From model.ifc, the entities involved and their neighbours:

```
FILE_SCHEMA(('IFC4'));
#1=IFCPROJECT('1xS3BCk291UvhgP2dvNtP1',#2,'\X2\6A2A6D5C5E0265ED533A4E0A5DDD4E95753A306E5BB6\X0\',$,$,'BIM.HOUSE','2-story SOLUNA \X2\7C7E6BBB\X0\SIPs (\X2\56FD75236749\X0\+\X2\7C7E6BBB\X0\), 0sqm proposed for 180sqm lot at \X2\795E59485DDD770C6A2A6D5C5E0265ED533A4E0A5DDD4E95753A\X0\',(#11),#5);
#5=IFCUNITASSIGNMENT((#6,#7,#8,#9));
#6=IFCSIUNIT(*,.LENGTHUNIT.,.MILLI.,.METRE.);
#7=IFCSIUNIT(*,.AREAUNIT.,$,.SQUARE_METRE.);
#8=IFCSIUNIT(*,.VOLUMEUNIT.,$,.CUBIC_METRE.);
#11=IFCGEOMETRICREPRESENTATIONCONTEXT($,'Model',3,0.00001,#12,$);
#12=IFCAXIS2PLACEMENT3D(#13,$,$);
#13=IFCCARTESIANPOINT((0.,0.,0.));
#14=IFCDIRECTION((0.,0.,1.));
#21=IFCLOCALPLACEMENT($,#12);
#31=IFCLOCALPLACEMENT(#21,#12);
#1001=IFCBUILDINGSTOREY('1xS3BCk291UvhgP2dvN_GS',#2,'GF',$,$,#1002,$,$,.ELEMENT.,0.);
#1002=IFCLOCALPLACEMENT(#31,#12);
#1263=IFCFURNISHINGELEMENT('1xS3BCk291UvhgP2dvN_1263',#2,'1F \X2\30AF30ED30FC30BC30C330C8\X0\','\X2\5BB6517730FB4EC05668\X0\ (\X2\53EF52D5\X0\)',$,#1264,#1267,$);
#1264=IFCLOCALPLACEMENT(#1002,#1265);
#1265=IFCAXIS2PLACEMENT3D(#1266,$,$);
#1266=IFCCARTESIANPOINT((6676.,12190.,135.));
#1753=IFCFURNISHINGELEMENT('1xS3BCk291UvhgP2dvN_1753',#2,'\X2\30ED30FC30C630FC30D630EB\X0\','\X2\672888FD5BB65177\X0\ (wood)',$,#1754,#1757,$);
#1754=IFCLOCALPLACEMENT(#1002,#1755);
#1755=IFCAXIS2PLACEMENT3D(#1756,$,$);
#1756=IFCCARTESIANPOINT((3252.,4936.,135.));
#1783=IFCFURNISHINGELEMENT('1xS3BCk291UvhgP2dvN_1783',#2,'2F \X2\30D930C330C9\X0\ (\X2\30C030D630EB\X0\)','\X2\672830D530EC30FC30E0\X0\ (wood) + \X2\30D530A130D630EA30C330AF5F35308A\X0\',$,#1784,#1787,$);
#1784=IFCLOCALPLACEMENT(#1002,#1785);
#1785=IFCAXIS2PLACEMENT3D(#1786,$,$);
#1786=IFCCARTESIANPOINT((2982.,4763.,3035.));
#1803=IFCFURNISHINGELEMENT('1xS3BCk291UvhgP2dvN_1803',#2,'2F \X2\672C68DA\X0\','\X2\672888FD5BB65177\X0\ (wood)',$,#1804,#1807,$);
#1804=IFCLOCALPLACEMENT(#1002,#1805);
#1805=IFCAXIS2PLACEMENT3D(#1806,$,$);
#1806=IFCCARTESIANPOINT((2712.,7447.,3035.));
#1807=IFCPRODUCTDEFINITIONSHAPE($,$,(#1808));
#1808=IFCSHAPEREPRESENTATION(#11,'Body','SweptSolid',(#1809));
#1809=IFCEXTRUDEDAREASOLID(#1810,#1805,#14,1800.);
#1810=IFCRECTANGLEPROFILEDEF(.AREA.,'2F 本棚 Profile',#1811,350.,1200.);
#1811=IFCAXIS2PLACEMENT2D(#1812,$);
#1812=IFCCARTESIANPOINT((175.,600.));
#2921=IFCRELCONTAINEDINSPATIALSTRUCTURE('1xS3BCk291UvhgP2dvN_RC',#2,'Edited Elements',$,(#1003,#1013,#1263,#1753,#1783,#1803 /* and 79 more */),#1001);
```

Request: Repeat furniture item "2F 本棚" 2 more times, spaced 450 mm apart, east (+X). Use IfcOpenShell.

```python
import numpy as np
import ifcopenshell
import ifcopenshell.api.geometry
import ifcopenshell.api.root
import ifcopenshell.util.element
import ifcopenshell.util.placement
import ifcopenshell.util.unit

model = ifcopenshell.open("model.ifc")
unit_scale = ifcopenshell.util.unit.calculate_unit_scale(model)


def reuse_history(source, copy):
    """copy_class also copies each property set's owner history, people and application; keep the originals."""
    for rel in copy.IsDefinedBy:
        if rel.is_a("IfcRelDefinesByProperties") and (history := rel.RelatingPropertyDefinition.OwnerHistory):
            rel.RelatingPropertyDefinition.OwnerHistory = source.OwnerHistory
            ifcopenshell.util.element.remove_deep2(model, history)


source = model.by_id(1803)
base = ifcopenshell.util.placement.get_local_placement(source.ObjectPlacement)
step = np.array([1.0, 0.0, 0.0]) * 0.45 / unit_scale

for i in range(1, 3):
    copy = ifcopenshell.api.root.copy_class(model, product=source)
    copy.Representation = ifcopenshell.util.element.copy_deep(
        model, source.Representation, exclude=["IfcGeometricRepresentationContext", "IfcRepresentationMap"]
    )
    reuse_history(source, copy)
    matrix = base.copy()
    matrix[:3, 3] += i * step
    print("added at", matrix[:3, 3].round(3) + 0.0)
    ifcopenshell.api.geometry.edit_object_placement(model, product=copy, matrix=matrix, is_si=False)

model.write("model_updated.ifc")
```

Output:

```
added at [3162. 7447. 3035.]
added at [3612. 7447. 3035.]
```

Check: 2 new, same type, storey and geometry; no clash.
